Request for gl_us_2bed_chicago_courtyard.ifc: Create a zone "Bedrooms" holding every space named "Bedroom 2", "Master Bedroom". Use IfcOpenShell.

First a look at what the model holds.

```python
import ifcopenshell

model = ifcopenshell.open("gl_us_2bed_chicago_courtyard.ifc")
print(model.schema)
seen = {}
for space in model.by_type("IfcSpace"):
    seen[space.LongName] = seen.get(space.LongName, 0) + 1
for name, count in sorted(seen.items(), key=str):
    print(count, "x", name)
print("zones:", [z.Name for z in model.by_type("IfcZone")][:20])
```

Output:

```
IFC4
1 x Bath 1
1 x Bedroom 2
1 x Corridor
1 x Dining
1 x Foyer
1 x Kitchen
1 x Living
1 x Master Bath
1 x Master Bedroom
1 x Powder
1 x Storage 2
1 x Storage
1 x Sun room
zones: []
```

```python
import ifcopenshell
import ifcopenshell.api.group
import ifcopenshell.api.root

model = ifcopenshell.open("gl_us_2bed_chicago_courtyard.ifc")

names = {"Bedroom 2", "Master Bedroom"}
spaces = [s for s in model.by_type("IfcSpace") if s.LongName in names]

zone = ifcopenshell.api.root.create_entity(model, ifc_class="IfcZone", name="Bedrooms")
ifcopenshell.api.group.assign_group(model, products=spaces, group=zone)
print(len(spaces), "spaces in", zone.Name)

model.write("gl_us_2bed_chicago_courtyard_edited.ifc")
```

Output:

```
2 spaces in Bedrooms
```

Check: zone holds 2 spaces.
